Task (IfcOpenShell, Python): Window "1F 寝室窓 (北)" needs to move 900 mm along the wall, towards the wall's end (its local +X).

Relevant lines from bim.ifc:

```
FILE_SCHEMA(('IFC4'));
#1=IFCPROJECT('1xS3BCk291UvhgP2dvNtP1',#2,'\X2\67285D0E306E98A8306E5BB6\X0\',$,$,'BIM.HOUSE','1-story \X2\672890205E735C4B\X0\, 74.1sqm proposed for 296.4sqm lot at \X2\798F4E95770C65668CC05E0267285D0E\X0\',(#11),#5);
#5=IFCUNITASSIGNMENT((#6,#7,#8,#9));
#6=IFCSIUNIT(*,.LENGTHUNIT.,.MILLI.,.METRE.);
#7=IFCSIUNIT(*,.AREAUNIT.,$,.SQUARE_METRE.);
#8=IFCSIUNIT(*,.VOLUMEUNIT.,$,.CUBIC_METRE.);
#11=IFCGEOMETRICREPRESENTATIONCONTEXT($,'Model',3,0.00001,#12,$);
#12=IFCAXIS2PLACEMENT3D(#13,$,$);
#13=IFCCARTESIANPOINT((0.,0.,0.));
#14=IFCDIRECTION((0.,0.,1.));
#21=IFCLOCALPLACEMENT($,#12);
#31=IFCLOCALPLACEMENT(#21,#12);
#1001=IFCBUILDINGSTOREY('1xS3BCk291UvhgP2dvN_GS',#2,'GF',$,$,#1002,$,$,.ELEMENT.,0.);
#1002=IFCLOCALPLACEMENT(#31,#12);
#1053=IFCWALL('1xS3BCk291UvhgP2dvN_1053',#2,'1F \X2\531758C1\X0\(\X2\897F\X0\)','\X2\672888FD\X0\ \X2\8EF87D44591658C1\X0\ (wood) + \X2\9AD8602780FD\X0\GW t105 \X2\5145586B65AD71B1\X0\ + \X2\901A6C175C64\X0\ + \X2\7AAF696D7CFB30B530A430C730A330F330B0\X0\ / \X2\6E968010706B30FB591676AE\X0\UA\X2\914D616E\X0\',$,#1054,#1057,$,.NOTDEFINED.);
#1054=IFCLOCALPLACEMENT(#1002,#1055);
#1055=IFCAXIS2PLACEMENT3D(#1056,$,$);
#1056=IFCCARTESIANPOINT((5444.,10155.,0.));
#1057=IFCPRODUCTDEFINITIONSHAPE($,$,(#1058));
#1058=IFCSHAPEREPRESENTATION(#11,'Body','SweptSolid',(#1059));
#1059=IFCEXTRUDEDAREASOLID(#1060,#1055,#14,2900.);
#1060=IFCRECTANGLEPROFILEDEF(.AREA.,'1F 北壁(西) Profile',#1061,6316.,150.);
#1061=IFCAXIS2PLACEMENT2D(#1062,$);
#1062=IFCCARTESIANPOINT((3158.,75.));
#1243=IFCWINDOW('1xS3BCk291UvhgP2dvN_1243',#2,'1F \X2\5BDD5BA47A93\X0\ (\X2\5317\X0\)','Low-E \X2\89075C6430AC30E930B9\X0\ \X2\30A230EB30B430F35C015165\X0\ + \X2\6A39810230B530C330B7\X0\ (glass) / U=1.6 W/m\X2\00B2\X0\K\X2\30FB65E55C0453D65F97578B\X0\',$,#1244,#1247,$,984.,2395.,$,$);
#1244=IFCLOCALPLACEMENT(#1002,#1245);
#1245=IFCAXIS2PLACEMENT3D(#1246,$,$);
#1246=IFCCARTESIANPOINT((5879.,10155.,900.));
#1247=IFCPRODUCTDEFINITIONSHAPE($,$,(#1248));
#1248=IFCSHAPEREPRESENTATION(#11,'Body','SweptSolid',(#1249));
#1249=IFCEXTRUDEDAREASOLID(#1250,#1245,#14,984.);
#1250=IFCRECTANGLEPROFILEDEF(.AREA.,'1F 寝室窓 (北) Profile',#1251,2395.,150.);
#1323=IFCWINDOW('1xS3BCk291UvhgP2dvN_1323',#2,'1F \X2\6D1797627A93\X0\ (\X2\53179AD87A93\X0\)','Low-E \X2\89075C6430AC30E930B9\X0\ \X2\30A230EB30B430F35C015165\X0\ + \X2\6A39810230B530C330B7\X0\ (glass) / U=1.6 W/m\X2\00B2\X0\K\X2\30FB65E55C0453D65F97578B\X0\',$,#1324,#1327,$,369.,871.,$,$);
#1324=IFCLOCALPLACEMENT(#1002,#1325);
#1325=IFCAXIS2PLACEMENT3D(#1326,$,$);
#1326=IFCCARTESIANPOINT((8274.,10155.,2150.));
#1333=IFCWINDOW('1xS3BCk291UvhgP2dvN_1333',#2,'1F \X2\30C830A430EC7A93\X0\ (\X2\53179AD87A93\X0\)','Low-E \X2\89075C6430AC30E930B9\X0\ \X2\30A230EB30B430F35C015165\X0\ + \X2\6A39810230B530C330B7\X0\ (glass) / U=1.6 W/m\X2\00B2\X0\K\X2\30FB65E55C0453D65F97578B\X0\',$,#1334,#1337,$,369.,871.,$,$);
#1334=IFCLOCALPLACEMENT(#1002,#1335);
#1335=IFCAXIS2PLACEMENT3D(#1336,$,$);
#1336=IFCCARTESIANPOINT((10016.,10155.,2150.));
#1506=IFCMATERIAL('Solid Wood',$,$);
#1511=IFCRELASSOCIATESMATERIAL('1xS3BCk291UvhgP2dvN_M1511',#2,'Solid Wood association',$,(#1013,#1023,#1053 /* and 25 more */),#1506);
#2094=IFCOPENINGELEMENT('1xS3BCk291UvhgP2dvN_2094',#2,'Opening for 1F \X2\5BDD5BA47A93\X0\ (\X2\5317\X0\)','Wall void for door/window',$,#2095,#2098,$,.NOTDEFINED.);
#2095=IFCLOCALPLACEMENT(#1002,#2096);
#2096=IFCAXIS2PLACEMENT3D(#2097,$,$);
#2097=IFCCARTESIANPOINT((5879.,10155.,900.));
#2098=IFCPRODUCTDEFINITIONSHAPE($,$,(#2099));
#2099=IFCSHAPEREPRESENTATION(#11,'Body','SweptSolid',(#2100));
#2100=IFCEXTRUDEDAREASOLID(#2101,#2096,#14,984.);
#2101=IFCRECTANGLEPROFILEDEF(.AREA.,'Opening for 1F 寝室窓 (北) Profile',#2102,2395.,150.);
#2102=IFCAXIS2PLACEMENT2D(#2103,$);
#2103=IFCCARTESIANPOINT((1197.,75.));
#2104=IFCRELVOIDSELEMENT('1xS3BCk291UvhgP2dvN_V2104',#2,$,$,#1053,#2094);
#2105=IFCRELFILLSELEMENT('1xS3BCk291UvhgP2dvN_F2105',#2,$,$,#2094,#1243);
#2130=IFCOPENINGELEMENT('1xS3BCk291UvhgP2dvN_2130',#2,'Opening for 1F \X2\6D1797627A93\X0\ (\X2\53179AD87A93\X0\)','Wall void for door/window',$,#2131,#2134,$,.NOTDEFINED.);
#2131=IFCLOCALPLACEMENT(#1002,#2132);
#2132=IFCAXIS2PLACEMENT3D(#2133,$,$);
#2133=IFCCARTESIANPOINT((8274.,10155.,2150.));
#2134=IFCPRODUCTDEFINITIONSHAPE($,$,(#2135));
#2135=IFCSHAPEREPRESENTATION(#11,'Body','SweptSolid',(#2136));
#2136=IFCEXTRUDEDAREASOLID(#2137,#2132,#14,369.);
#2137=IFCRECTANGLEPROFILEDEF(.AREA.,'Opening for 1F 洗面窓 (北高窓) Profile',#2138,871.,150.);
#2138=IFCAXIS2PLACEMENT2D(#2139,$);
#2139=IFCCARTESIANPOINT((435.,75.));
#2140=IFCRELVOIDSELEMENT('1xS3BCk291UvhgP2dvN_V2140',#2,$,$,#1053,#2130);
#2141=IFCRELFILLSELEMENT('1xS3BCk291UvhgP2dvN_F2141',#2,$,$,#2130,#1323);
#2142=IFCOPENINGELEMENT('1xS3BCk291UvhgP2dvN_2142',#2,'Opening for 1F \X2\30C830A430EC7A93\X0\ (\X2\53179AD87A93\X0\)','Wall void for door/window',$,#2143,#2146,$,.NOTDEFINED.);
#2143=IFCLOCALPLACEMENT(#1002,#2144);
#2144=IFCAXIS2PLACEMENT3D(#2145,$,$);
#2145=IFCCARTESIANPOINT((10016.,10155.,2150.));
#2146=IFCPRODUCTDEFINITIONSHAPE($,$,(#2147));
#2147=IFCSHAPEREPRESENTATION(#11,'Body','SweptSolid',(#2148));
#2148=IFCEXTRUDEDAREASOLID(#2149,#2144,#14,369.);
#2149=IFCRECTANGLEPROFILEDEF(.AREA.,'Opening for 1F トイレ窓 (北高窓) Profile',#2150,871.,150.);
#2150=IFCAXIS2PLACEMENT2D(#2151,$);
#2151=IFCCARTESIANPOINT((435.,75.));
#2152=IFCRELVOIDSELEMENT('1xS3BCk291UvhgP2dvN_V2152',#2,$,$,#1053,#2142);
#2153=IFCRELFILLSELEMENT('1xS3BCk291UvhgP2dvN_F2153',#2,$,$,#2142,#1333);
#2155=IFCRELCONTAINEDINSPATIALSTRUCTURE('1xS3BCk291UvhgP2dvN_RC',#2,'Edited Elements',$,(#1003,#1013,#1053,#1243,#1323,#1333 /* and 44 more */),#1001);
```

```python
import ifcopenshell
import ifcopenshell.api.geometry
import ifcopenshell.util.placement

model = ifcopenshell.open("bim.ifc")

window = model.by_guid("1xS3BCk291UvhgP2dvN_1243")
opening = window.FillsVoids[0].RelatingOpeningElement
wall = opening.VoidsElements[0].RelatingBuildingElement

wall_matrix = ifcopenshell.util.placement.get_local_placement(wall.ObjectPlacement)
shift = wall_matrix[:3, 0] * 900.0
before = ifcopenshell.util.placement.get_local_placement(window.ObjectPlacement)[:3, 3].copy()

# The window is not placed relative to its opening, so move both.
for product in (opening, window):
    matrix = ifcopenshell.util.placement.get_local_placement(product.ObjectPlacement)
    matrix[:3, 3] += shift
    ifcopenshell.api.geometry.edit_object_placement(model, product=product, matrix=matrix, is_si=False)

after = ifcopenshell.util.placement.get_local_placement(window.ObjectPlacement)[:3, 3]
print("window moved by", (after - before).round(3) + 0.0)

model.write("bim_updated.ifc")
```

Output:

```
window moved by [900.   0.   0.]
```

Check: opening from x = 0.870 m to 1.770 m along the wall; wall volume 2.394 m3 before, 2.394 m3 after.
